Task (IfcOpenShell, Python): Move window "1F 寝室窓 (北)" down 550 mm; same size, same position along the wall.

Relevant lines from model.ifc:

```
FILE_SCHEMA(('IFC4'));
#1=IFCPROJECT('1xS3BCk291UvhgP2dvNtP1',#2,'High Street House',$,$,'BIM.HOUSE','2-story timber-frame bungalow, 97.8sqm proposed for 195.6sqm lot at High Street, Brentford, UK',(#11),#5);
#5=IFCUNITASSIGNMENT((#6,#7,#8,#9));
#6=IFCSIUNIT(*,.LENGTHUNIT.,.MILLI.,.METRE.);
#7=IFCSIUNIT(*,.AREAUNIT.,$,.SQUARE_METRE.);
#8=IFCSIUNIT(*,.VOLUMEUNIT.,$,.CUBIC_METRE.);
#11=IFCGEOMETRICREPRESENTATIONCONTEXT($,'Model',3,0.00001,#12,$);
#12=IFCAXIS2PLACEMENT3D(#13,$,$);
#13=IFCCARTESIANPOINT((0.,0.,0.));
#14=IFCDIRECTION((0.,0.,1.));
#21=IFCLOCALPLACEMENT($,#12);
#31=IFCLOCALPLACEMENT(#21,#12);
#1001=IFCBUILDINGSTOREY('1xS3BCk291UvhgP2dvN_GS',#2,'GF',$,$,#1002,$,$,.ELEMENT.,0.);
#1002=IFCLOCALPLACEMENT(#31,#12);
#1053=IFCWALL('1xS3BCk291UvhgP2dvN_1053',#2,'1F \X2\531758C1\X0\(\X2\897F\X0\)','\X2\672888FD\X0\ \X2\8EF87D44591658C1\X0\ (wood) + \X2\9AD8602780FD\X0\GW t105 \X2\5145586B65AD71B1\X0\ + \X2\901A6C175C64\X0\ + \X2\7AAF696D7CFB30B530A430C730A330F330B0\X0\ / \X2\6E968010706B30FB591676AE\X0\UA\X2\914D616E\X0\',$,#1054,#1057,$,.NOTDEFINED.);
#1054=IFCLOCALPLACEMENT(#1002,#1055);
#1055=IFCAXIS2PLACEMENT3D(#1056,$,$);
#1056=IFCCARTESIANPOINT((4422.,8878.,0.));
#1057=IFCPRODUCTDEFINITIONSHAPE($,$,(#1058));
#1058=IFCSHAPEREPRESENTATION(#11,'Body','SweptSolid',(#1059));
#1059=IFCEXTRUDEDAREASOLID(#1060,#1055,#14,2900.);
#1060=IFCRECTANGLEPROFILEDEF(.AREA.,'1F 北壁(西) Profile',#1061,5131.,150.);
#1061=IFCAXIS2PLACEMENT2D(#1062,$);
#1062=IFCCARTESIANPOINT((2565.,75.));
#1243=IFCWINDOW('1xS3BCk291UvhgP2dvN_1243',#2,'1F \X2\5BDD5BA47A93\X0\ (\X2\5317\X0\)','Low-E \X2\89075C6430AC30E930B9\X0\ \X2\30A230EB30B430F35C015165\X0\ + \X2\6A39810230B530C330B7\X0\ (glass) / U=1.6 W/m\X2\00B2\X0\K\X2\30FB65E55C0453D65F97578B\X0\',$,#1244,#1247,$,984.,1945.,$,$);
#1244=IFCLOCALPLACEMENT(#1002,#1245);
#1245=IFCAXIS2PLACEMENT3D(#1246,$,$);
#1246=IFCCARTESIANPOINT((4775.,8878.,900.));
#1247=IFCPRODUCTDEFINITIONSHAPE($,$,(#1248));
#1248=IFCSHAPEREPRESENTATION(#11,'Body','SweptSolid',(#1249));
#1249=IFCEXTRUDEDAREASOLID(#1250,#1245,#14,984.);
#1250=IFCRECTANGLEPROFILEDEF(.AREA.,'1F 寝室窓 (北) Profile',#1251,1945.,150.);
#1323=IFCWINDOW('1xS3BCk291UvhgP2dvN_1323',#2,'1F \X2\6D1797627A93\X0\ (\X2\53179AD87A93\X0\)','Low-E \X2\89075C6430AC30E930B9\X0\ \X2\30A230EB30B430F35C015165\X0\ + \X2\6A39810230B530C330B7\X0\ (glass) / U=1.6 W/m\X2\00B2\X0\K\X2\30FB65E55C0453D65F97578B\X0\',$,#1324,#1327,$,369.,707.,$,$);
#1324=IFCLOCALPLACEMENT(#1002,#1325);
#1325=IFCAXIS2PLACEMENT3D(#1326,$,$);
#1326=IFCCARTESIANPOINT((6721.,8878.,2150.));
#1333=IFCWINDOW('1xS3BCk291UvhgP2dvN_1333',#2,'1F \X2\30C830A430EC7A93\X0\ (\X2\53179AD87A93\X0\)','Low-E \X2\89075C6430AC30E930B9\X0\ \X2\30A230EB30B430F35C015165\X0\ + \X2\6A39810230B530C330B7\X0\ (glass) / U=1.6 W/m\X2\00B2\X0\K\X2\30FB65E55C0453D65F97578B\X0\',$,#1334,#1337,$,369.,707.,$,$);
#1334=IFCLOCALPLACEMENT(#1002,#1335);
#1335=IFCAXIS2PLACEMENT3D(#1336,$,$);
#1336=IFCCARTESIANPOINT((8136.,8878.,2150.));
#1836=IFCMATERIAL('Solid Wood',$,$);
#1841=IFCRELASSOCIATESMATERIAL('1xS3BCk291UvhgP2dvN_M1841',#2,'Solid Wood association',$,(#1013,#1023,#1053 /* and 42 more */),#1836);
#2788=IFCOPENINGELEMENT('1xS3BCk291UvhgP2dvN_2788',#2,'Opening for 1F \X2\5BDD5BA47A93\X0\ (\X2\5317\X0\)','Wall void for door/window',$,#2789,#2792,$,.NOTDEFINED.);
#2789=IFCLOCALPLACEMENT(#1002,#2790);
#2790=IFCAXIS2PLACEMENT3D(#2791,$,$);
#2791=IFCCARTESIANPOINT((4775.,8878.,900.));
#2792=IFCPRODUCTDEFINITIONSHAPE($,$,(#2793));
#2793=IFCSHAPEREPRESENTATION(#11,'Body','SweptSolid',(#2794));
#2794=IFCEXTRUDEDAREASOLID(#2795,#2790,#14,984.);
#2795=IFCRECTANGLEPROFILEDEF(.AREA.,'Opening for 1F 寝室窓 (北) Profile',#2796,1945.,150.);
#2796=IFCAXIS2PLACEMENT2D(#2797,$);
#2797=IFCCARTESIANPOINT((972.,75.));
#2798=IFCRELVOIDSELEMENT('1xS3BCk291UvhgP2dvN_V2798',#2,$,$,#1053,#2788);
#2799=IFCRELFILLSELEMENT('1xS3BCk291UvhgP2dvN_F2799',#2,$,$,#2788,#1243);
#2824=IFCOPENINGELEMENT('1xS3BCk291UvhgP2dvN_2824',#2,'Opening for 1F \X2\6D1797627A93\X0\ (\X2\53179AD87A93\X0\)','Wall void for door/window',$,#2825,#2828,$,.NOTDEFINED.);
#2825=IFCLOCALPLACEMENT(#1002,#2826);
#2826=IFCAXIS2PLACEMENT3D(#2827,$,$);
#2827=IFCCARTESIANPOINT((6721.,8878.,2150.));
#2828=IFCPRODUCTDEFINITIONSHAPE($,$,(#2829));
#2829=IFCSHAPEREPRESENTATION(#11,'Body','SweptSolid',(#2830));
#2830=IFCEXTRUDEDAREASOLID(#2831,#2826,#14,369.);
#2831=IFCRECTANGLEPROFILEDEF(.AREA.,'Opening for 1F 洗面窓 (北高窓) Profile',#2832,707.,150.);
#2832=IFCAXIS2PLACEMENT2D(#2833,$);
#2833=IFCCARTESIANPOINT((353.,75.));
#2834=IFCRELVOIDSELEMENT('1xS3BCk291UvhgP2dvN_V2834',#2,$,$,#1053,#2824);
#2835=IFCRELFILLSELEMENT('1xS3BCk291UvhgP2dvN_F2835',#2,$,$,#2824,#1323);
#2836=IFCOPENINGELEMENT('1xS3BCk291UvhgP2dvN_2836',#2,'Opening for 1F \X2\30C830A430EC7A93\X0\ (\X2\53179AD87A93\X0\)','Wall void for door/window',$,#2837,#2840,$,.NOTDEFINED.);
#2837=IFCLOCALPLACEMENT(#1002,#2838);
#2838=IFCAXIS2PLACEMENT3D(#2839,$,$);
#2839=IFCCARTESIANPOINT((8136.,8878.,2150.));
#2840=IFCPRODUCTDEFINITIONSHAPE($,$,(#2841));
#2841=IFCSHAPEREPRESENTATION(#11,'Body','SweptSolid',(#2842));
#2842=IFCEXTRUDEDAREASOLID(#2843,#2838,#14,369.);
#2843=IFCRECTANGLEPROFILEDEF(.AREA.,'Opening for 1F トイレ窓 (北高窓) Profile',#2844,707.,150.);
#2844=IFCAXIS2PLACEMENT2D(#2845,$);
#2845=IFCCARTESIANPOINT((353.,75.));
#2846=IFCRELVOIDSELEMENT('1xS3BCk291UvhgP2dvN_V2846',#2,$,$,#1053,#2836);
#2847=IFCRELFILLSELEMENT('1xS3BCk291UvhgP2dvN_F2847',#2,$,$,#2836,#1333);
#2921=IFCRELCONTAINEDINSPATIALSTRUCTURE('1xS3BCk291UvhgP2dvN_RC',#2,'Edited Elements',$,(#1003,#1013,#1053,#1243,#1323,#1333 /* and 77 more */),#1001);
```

```python
import numpy as np
import ifcopenshell
import ifcopenshell.api.geometry
import ifcopenshell.util.placement
import ifcopenshell.util.unit

model = ifcopenshell.open("model.ifc")
unit_scale = ifcopenshell.util.unit.calculate_unit_scale(model)

window = model.by_guid("1xS3BCk291UvhgP2dvN_1243")
opening = window.FillsVoids[0].RelatingOpeningElement
dz = -550.0

shift = np.array([0.0, 0.0, dz])
# The window is not placed relative to its opening, so move both.
for product in (opening, window):
    matrix = ifcopenshell.util.placement.get_local_placement(product.ObjectPlacement)
    matrix[:3, 3] += shift
    ifcopenshell.api.geometry.edit_object_placement(model, product=product, matrix=matrix, is_si=False)

print(f"moved by {dz * unit_scale:+.3f} m")

model.write("model_v2.ifc")
```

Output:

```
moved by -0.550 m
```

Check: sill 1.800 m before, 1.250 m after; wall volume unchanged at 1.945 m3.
